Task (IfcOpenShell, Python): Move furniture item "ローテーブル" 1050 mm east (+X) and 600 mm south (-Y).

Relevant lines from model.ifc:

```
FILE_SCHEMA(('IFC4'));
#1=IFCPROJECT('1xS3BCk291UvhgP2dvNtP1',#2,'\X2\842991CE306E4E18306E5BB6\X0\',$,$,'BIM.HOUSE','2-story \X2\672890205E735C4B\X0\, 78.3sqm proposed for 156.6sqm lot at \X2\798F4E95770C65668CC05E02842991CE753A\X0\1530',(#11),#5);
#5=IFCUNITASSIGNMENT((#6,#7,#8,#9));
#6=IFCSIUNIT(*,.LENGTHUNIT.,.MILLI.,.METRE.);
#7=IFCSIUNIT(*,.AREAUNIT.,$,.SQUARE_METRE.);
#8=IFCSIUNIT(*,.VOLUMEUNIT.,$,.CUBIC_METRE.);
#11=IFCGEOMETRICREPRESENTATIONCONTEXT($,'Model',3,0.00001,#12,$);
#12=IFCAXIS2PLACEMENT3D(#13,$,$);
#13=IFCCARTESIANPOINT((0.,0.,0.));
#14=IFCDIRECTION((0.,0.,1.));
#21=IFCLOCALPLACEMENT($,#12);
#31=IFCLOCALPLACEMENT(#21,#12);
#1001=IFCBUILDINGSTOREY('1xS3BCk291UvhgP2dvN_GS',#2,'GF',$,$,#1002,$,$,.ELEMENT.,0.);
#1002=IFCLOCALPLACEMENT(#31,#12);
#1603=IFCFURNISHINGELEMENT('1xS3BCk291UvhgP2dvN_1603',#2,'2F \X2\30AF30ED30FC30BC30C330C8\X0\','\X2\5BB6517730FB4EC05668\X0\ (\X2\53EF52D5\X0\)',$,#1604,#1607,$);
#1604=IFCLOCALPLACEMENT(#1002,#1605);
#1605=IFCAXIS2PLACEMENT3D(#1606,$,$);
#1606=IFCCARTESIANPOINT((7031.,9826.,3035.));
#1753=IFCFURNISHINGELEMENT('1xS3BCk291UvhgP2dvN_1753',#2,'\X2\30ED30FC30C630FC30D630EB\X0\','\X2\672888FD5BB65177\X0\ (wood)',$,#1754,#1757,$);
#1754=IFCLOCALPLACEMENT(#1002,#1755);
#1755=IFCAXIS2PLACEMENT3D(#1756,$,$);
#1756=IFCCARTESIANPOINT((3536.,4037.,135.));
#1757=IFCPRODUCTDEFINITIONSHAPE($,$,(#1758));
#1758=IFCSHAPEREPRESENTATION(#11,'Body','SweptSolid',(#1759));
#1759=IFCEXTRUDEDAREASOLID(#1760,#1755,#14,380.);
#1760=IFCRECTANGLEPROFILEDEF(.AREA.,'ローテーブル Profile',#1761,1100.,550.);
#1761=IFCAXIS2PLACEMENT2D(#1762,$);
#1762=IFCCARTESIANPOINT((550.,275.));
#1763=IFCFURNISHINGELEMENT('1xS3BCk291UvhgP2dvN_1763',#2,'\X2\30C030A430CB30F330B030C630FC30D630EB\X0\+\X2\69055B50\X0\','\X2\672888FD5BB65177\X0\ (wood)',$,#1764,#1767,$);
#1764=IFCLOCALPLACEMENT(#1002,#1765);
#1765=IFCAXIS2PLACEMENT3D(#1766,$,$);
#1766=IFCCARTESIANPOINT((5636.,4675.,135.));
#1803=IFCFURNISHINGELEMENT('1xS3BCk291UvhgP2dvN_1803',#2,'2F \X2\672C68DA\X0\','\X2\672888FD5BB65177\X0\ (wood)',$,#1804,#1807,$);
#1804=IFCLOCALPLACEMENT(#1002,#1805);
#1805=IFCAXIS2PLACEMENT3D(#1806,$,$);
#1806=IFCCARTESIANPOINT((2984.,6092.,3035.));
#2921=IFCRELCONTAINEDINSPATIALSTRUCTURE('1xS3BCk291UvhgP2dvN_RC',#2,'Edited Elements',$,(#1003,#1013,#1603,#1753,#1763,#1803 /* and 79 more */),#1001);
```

```python
import ifcopenshell
import ifcopenshell.api.geometry
import ifcopenshell.util.placement

model = ifcopenshell.open("model.ifc")

item = model.by_id(1753)
matrix = ifcopenshell.util.placement.get_local_placement(item.ObjectPlacement)
matrix[0, 3] += 1050.0
matrix[1, 3] -= 600.0
ifcopenshell.api.geometry.edit_object_placement(model, product=item, matrix=matrix, is_si=False)

print(ifcopenshell.util.placement.get_local_placement(item.ObjectPlacement).round(3) + 0.0)

model.write("model_edited.ifc")
```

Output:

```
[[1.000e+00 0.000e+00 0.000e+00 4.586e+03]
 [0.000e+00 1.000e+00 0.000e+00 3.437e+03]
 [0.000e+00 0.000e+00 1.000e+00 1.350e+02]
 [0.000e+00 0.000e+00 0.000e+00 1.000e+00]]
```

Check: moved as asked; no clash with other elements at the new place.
